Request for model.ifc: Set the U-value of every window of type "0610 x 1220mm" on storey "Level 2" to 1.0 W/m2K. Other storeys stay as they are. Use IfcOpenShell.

First a look at what the model holds.

```python
import ifcopenshell
import ifcopenshell.util.element

model = ifcopenshell.open("model.ifc")
print(model.schema)
storey = next(s for s in model.by_type("IfcBuildingStorey") if s.Name == "Level 2")
windows = [e for e in ifcopenshell.util.element.get_decomposition(storey) if e.is_a("IfcWindow")]
seen = {}
for e in windows:
    element_type = ifcopenshell.util.element.get_type(e)
    key = (element_type.Name if element_type != e and element_type else None, ifcopenshell.util.element.get_pset(e, "Pset_WindowCommon", "ThermalTransmittance"))
    seen[key] = seen.get(key, 0) + 1
for (name, value), count in sorted(seen.items(), key=str):
    print(count, "x", name, "|", value)
```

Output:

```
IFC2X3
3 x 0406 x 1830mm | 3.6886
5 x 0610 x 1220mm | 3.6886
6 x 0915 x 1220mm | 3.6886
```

```python
import ifcopenshell
import ifcopenshell.api.pset
import ifcopenshell.util.element

model = ifcopenshell.open("model.ifc")

storey = next(s for s in model.by_type("IfcBuildingStorey") if s.Name == "Level 2")
windows = [e for e in ifcopenshell.util.element.get_decomposition(storey) if e.is_a("IfcWindow")]

count = 0
for e in windows:
    element_type = ifcopenshell.util.element.get_type(e)
    if element_type in (None, e) or element_type.Name != "0610 x 1220mm":
        continue
    # add_pset returns the element's existing set when there is one.
    pset = ifcopenshell.api.pset.add_pset(model, product=e, name="Pset_WindowCommon")
    ifcopenshell.api.pset.edit_pset(model, pset=pset, properties={"ThermalTransmittance": 1.0})
    count += 1

print(count, "windows updated")

model.write("model_edited.ifc")
```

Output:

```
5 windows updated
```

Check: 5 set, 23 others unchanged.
